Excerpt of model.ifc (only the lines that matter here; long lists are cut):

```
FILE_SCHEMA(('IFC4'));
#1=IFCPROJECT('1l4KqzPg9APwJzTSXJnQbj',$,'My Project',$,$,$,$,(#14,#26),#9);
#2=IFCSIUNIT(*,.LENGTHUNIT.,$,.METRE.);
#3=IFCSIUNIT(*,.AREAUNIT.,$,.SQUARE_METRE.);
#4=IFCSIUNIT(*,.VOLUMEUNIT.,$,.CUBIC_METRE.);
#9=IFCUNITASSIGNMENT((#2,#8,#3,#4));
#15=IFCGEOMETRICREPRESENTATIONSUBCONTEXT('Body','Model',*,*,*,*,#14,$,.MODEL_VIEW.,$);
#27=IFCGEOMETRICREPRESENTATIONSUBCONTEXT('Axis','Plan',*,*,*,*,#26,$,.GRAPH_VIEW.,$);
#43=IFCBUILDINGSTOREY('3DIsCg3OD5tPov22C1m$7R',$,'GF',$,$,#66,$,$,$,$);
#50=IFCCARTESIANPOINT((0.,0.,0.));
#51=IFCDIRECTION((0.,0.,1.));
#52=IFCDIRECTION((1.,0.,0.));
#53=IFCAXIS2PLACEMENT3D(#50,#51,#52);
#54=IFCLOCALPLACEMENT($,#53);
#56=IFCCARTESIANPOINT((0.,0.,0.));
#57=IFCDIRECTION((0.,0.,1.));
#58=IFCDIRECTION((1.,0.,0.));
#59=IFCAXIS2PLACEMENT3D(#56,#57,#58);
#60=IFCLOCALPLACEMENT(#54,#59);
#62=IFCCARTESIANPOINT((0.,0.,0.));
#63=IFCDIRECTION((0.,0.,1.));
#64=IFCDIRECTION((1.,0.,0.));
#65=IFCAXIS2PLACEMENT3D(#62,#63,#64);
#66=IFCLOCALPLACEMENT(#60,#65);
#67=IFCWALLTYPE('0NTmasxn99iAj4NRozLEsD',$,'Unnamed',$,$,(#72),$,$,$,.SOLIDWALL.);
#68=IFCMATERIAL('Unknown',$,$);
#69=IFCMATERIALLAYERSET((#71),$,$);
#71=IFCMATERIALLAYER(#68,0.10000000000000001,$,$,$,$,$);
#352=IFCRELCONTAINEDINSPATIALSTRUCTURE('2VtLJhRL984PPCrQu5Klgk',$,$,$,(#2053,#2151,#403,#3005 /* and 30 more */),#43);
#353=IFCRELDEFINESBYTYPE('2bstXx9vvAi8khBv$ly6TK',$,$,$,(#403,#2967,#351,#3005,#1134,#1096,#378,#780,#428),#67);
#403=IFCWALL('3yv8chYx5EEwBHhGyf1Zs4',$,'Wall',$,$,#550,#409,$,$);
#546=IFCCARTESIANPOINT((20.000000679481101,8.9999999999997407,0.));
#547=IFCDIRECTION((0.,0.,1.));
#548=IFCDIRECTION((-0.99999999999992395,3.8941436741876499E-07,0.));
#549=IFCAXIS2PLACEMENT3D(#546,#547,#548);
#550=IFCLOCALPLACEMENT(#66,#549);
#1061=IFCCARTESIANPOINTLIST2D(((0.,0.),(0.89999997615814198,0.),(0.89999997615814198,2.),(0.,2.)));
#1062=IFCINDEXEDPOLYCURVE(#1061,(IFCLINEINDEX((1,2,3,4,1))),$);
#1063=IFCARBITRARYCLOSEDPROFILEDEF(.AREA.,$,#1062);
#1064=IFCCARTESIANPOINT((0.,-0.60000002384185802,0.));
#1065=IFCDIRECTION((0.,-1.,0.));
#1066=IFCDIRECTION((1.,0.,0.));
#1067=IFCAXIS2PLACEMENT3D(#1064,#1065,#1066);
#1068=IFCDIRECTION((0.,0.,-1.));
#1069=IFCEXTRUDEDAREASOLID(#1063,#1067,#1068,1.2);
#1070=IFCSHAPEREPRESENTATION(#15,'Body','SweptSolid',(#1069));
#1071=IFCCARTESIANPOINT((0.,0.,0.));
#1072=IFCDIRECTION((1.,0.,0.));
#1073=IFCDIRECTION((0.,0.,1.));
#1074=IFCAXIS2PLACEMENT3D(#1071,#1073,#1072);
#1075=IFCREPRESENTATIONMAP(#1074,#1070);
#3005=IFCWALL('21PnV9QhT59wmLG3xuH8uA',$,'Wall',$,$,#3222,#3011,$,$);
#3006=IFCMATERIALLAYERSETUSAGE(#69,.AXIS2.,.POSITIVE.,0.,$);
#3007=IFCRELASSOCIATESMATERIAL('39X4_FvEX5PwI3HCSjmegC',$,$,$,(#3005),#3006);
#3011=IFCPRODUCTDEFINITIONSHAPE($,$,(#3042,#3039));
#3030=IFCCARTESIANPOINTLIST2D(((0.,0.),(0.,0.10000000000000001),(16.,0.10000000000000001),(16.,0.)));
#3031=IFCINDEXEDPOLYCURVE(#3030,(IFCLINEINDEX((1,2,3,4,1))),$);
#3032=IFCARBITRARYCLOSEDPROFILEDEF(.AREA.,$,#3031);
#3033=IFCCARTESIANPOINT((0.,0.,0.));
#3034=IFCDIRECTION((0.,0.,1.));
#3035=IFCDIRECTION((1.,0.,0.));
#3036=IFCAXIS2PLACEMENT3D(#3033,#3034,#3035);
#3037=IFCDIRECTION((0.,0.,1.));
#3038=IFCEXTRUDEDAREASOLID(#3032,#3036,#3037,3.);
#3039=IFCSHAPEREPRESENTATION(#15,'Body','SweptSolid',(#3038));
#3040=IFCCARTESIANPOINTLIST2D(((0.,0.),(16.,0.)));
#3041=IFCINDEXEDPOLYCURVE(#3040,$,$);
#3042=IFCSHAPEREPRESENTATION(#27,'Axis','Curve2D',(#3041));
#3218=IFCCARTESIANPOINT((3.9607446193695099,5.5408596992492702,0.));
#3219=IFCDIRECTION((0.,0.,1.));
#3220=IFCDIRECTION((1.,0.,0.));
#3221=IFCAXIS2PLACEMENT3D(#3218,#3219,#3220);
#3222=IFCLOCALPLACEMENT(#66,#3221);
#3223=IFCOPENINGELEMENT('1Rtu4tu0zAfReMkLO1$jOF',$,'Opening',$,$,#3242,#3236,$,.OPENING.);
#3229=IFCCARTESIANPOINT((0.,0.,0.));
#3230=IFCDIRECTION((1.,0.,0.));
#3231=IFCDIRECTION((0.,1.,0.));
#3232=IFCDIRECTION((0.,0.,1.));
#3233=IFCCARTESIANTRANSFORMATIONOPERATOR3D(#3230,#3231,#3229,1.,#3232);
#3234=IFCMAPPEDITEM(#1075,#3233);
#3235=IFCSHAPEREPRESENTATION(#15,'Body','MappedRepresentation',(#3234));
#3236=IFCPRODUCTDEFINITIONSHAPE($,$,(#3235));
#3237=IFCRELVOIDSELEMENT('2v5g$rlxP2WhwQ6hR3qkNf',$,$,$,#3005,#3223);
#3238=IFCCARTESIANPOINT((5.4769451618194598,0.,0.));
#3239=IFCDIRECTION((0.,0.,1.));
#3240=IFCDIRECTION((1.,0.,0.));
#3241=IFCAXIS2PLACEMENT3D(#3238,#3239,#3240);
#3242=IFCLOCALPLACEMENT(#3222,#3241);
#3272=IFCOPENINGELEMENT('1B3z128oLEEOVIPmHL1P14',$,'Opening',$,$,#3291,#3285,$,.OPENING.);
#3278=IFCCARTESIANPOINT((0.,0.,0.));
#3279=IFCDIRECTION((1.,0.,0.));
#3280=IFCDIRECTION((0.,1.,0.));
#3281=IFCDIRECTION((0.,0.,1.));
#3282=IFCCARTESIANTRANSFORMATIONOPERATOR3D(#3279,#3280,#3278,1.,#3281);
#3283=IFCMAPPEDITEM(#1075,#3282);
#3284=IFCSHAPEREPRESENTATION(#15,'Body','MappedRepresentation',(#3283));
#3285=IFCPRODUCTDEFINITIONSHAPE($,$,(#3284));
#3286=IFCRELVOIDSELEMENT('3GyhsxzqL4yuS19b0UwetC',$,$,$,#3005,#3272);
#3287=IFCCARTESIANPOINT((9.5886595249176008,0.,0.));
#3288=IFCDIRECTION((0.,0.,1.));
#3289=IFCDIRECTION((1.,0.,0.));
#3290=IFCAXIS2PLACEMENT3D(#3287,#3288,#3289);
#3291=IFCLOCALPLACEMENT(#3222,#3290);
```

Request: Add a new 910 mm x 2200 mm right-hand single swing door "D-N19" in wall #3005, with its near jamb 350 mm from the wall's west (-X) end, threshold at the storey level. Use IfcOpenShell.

```python
import numpy as np
import ifcopenshell
import ifcopenshell.api.feature
import ifcopenshell.api.geometry
import ifcopenshell.api.root
import ifcopenshell.api.spatial
import ifcopenshell.geom
import ifcopenshell.util.element
import ifcopenshell.util.placement
import ifcopenshell.util.representation
import ifcopenshell.util.shape
import ifcopenshell.util.unit

model = ifcopenshell.open("model.ifc")
unit_scale = ifcopenshell.util.unit.calculate_unit_scale(model)
settings = ifcopenshell.geom.settings()


def volume(element):
    """Net volume in cubic metres, openings subtracted."""
    shape = ifcopenshell.geom.create_shape(settings, element)
    return ifcopenshell.util.shape.get_volume(shape.geometry)


wall = model.by_id(3005)
storey = ifcopenshell.util.element.get_container(wall, ifc_class="IfcBuildingStorey")
context = ifcopenshell.util.representation.get_context(model, "Model", "Body", "MODEL_VIEW")
before = volume(wall)

width, height, from_end, sill = 0.91, 2.2, 0.35, 0.0  # metres

# The wall runs along its own X axis, and the end named is its -X end.
wall_shape = ifcopenshell.geom.create_shape(settings, wall)
x, y, z = ifcopenshell.util.shape.get_vertices(wall_shape.geometry).T
start = x.min() + from_end
face, thickness = float(y.min()), float(y.max() - y.min())
wall_matrix = ifcopenshell.util.placement.get_local_placement(wall.ObjectPlacement)
level = ifcopenshell.util.placement.get_local_placement(storey.ObjectPlacement)[2, 3]


def in_wall(x, y):
    """Placement at x, y metres in the wall's axes, at sill height."""
    matrix = wall_matrix.copy()
    matrix[:, 3] = wall_matrix @ np.array([x / unit_scale, y / unit_scale, 0.0, 1.0])
    matrix[2, 3] = level + sill / unit_scale
    return matrix


# Opening: a box that overshoots both wall faces by 50 mm.
opening = ifcopenshell.api.root.create_entity(model, ifc_class="IfcOpeningElement", predefined_type="OPENING")
box = ifcopenshell.api.geometry.add_wall_representation(
    model, context=context, length=width, height=height, thickness=thickness + 0.1
)
ifcopenshell.api.geometry.assign_representation(model, product=opening, representation=box)
ifcopenshell.api.geometry.edit_object_placement(model, product=opening, matrix=in_wall(start, face - 0.05), is_si=False)
ifcopenshell.api.feature.add_feature(model, feature=opening, element=wall)

door = ifcopenshell.api.root.create_entity(model, ifc_class="IfcDoor", name="D-N19", predefined_type="DOOR")
door.OverallWidth, door.OverallHeight = width / unit_scale, height / unit_scale
door.OperationType = "SINGLE_SWING_RIGHT"
body = ifcopenshell.api.geometry.add_door_representation(
    model,
    context=context,
    overall_width=door.OverallWidth,
    overall_height=door.OverallHeight,
    operation_type="SINGLE_SWING_RIGHT",
    lining_properties={"LiningDepth": thickness / unit_scale, "ThresholdDepth": thickness / unit_scale},
)
ifcopenshell.api.geometry.assign_representation(model, product=door, representation=body)
ifcopenshell.api.spatial.assign_container(model, products=[door], relating_structure=storey)
ifcopenshell.api.feature.add_filling(model, opening=opening, element=door)

# The lining spans the wall, so the door starts at the wall face.
ifcopenshell.api.geometry.edit_object_placement(model, product=door, matrix=in_wall(start, face), is_si=False)

after = volume(wall)

print(f"wall volume {before:.3f} -> {after:.3f} m3")

model.write("model_rev.ifc")
```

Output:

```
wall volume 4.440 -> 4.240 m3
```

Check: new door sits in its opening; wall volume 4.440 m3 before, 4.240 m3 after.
